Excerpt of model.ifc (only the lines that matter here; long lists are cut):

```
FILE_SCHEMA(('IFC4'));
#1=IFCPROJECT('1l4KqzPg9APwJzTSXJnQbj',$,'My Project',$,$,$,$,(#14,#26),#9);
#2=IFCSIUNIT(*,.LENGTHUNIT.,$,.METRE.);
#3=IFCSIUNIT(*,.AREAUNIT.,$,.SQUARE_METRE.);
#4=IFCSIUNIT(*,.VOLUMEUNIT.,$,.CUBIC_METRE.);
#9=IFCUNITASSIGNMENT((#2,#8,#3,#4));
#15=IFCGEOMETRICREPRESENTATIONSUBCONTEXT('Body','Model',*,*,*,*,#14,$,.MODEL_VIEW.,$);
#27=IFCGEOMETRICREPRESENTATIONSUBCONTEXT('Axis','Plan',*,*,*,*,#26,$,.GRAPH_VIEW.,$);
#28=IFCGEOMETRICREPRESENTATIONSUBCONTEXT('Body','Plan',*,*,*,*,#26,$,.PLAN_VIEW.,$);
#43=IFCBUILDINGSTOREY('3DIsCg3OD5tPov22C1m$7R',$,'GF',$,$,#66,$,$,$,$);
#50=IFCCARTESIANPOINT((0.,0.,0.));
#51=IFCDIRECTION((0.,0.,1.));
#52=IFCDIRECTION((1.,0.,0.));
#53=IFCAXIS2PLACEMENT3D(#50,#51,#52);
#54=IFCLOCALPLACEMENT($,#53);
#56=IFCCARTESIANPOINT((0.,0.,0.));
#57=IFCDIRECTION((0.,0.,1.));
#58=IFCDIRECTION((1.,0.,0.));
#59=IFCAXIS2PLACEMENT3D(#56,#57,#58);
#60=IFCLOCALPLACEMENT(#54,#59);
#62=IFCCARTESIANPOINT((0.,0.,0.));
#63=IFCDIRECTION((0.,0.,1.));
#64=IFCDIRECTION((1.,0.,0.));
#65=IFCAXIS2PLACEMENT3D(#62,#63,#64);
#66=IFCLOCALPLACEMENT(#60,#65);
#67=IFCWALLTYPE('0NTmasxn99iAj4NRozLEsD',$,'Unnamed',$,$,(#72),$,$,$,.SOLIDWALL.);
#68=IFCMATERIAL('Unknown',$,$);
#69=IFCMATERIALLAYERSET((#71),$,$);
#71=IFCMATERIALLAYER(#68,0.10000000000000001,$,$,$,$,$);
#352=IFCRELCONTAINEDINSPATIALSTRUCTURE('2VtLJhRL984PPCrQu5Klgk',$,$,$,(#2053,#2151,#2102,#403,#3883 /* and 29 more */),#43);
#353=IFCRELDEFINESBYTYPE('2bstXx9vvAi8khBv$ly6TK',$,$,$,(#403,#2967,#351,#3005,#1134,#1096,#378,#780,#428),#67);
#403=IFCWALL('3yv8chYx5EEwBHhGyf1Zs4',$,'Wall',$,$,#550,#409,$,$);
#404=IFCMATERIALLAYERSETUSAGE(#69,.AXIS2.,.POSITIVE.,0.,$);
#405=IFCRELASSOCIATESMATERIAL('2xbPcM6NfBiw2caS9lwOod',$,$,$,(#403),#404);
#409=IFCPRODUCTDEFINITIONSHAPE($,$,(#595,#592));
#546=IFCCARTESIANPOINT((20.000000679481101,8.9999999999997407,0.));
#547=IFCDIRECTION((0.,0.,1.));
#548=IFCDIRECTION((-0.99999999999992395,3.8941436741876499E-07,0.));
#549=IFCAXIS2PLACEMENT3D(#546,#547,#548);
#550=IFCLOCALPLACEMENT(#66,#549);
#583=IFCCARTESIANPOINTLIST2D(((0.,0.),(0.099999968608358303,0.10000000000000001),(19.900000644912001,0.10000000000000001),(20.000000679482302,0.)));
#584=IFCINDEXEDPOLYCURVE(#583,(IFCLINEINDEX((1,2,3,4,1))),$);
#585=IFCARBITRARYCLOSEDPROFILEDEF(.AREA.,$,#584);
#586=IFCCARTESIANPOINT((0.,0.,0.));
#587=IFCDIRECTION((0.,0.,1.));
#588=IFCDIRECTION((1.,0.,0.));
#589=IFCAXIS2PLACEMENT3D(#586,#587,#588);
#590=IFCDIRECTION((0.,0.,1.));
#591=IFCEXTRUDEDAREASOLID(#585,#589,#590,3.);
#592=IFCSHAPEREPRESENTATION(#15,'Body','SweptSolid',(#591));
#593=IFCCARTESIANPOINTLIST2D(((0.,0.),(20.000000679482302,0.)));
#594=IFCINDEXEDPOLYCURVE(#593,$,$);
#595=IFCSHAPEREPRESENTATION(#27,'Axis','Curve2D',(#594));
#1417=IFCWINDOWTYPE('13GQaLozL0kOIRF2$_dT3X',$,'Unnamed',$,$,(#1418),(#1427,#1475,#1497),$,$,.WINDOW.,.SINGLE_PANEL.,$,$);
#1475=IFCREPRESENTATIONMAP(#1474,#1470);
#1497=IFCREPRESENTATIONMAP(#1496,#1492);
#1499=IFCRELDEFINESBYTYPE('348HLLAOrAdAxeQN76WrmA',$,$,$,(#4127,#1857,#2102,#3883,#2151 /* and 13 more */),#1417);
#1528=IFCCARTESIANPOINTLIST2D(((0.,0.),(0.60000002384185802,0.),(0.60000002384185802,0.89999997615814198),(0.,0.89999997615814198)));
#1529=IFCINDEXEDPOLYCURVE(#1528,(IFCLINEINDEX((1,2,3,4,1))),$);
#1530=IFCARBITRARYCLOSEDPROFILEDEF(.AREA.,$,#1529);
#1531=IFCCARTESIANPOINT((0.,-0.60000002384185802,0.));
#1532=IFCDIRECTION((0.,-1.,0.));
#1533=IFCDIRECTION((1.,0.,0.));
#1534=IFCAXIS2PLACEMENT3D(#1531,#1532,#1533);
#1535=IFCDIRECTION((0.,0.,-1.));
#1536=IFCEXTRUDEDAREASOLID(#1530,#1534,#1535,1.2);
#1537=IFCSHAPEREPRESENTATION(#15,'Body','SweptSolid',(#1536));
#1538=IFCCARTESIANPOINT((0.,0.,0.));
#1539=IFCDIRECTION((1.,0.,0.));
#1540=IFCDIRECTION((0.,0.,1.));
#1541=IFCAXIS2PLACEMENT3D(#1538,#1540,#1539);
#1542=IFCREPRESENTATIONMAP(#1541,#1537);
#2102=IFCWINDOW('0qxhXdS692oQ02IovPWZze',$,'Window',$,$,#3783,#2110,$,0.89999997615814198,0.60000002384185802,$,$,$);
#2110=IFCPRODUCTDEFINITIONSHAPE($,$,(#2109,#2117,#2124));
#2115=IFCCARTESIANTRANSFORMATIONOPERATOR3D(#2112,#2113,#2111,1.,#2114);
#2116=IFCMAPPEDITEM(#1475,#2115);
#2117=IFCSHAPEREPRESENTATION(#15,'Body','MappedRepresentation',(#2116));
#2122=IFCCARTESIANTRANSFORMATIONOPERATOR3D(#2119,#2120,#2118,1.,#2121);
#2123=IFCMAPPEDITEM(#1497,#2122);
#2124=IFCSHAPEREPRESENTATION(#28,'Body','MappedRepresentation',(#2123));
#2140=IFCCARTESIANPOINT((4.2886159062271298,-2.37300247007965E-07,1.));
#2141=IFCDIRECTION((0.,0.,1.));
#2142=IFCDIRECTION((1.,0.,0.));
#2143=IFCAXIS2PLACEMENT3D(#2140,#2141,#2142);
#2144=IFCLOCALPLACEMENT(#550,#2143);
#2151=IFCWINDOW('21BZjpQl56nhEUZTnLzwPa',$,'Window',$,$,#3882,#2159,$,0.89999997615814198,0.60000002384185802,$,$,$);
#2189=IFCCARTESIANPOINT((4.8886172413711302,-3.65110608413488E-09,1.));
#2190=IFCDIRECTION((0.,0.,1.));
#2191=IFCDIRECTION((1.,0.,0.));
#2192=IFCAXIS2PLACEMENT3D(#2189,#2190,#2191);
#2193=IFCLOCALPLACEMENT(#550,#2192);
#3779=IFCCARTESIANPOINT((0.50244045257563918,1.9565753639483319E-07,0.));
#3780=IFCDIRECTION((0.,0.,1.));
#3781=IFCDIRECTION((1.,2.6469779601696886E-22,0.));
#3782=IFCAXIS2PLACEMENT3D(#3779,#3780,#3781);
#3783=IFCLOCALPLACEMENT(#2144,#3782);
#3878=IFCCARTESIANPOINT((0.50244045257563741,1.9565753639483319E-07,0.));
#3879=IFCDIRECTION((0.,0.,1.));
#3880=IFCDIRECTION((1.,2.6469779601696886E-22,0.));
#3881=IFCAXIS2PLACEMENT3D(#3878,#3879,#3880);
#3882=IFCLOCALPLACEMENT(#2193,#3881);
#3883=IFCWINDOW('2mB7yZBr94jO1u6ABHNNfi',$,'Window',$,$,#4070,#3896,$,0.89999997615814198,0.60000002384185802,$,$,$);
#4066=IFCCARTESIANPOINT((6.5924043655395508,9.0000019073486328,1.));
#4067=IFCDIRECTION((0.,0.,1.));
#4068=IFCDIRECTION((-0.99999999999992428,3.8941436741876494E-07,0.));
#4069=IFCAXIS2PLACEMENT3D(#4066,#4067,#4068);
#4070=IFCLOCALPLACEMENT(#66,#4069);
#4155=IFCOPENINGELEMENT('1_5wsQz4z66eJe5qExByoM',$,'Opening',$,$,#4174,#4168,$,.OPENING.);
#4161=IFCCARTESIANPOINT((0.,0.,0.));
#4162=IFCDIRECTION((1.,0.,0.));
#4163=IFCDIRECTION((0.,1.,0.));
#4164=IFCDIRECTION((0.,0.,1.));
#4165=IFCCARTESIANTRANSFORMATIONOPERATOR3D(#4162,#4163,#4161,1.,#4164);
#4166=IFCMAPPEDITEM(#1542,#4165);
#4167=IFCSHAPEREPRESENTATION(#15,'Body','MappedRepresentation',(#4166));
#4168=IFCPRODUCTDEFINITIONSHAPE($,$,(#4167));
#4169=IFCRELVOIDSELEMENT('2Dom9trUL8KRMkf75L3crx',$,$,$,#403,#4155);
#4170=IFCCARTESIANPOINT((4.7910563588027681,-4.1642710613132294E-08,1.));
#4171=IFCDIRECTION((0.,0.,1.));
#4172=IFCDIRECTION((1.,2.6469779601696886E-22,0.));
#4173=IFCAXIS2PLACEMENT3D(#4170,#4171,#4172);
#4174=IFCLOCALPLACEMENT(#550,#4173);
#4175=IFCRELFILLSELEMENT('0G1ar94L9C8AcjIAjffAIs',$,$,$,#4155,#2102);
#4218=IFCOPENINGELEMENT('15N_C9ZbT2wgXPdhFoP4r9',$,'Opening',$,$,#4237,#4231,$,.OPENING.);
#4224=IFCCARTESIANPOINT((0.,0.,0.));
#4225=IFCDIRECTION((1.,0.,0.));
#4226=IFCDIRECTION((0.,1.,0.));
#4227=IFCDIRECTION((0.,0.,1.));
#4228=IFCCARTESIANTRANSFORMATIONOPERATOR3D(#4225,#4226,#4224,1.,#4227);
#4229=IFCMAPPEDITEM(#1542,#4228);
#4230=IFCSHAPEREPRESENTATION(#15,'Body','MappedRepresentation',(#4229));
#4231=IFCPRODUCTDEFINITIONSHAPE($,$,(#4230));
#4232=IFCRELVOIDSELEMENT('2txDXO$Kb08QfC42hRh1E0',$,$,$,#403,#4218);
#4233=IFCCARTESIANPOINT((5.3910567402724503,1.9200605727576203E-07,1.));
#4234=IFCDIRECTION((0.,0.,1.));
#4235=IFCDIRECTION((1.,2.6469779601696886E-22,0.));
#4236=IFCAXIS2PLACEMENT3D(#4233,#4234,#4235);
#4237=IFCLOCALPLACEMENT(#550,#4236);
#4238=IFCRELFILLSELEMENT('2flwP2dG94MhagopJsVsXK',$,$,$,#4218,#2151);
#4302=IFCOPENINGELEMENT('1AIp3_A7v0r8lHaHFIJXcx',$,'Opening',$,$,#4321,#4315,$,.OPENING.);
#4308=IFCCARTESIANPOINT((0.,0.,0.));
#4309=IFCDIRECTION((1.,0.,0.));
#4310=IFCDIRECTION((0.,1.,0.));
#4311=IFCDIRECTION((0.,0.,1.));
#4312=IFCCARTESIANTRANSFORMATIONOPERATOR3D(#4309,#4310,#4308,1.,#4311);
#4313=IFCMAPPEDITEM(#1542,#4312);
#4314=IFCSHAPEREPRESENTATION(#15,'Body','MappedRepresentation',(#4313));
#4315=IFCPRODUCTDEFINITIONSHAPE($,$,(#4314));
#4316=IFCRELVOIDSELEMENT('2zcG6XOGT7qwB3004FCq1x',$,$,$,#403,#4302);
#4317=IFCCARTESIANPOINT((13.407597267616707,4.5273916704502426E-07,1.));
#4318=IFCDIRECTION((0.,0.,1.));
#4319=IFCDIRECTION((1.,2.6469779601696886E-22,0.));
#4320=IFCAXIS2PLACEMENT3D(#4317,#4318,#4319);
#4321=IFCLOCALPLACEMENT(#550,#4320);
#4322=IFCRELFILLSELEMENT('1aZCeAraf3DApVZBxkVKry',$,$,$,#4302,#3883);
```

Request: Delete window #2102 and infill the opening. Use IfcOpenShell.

```python
import ifcopenshell
import ifcopenshell.api.feature
import ifcopenshell.api.root
import ifcopenshell.geom
import ifcopenshell.util.shape

model = ifcopenshell.open("model.ifc")
settings = ifcopenshell.geom.settings()


def volume(element):
    """Net volume in cubic metres, openings subtracted."""
    shape = ifcopenshell.geom.create_shape(settings, element)
    return ifcopenshell.util.shape.get_volume(shape.geometry)


window = model.by_guid("0qxhXdS692oQ02IovPWZze")
opening = window.FillsVoids[0].RelatingOpeningElement
wall = opening.VoidsElements[0].RelatingBuildingElement
before = volume(wall)

ifcopenshell.api.root.remove_product(model, product=window)
ifcopenshell.api.feature.remove_feature(model, feature=opening)

after = volume(wall)

print(f"wall volume {before:.3f} -> {after:.3f} m3")

model.write("model-out.ifc")
```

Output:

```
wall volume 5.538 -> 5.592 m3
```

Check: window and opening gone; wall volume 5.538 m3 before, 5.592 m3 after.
